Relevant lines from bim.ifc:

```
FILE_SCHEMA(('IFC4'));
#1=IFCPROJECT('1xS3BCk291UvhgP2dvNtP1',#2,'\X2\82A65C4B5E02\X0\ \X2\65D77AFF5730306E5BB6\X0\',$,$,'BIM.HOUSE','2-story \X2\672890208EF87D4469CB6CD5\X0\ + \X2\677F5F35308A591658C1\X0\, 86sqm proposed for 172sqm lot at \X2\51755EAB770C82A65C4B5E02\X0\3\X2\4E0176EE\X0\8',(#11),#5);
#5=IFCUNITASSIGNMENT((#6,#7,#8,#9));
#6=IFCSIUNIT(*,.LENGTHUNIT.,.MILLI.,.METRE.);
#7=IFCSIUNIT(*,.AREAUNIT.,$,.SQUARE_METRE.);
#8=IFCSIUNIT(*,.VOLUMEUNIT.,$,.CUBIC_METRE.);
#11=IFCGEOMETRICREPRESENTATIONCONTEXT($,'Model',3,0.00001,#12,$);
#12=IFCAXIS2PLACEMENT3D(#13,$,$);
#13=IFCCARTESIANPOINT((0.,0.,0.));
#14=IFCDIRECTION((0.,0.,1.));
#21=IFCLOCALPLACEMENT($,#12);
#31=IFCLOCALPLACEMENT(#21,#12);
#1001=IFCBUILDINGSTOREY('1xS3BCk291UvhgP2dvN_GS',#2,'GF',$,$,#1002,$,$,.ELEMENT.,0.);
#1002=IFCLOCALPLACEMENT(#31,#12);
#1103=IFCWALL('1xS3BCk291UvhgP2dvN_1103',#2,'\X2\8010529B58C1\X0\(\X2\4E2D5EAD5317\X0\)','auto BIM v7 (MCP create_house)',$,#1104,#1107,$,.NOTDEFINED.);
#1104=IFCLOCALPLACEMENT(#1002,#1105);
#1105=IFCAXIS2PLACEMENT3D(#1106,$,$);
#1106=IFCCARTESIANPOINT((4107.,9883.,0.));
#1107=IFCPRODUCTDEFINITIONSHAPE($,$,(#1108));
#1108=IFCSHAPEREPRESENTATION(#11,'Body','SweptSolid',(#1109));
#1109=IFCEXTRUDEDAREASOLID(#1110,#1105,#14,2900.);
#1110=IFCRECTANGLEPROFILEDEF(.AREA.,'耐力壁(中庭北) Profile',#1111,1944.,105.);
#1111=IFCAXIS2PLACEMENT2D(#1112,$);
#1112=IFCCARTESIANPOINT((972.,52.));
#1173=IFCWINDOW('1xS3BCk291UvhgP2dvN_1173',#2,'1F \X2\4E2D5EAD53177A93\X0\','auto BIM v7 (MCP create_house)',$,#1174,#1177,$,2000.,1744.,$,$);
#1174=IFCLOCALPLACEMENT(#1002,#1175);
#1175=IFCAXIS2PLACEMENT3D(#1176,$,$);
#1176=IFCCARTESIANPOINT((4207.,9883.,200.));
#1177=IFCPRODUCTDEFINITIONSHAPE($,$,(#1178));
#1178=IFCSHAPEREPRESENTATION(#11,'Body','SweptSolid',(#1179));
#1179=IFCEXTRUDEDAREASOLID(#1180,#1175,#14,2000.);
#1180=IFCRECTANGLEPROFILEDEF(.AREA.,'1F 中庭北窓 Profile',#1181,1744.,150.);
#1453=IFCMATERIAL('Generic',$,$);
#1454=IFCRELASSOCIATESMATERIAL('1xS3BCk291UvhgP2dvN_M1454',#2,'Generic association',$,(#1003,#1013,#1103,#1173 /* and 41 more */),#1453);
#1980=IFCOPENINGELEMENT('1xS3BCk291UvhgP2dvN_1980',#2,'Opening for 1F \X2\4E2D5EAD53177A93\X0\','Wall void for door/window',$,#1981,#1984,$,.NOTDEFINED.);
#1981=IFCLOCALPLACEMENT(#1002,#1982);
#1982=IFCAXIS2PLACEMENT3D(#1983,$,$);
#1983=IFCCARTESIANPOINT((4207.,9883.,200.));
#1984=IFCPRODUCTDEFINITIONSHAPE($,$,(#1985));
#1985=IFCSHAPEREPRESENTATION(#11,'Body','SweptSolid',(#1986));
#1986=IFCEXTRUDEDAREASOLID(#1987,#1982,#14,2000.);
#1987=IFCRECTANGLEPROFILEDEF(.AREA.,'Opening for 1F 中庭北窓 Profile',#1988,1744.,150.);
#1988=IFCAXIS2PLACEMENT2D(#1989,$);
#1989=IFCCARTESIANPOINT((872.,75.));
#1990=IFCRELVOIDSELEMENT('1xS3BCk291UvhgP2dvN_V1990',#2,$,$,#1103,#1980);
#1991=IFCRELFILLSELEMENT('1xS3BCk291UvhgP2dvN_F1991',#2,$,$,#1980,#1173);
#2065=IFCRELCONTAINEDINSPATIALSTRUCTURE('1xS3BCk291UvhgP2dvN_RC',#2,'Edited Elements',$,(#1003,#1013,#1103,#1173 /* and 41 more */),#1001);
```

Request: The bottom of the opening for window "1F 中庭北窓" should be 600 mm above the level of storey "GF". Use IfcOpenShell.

```python
import numpy as np
import ifcopenshell
import ifcopenshell.api.geometry
import ifcopenshell.geom
import ifcopenshell.util.element
import ifcopenshell.util.placement
import ifcopenshell.util.shape
import ifcopenshell.util.unit

model = ifcopenshell.open("bim.ifc")
unit_scale = ifcopenshell.util.unit.calculate_unit_scale(model)

window = model.by_guid("1xS3BCk291UvhgP2dvN_1173")
opening = window.FillsVoids[0].RelatingOpeningElement
storey = ifcopenshell.util.element.get_container(window, ifc_class="IfcBuildingStorey")
level = ifcopenshell.util.placement.get_local_placement(storey.ObjectPlacement)[2, 3]

# The opening's origin need not be at the sill, so measure its lowest point.
shape = ifcopenshell.geom.create_shape(ifcopenshell.geom.settings(), opening)
bottom = ifcopenshell.util.shape.get_shape_bottom_elevation(shape, shape.geometry) / unit_scale
dz = level + 0.6 / unit_scale - bottom

shift = np.array([0.0, 0.0, dz])
# The window is not placed relative to its opening, so move both.
for product in (opening, window):
    matrix = ifcopenshell.util.placement.get_local_placement(product.ObjectPlacement)
    matrix[:3, 3] += shift
    ifcopenshell.api.geometry.edit_object_placement(model, product=product, matrix=matrix, is_si=False)

print(f"moved by {dz * unit_scale:+.3f} m")

model.write("bim_rev.ifc")
```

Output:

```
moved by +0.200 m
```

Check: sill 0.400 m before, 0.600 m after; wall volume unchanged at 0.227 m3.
